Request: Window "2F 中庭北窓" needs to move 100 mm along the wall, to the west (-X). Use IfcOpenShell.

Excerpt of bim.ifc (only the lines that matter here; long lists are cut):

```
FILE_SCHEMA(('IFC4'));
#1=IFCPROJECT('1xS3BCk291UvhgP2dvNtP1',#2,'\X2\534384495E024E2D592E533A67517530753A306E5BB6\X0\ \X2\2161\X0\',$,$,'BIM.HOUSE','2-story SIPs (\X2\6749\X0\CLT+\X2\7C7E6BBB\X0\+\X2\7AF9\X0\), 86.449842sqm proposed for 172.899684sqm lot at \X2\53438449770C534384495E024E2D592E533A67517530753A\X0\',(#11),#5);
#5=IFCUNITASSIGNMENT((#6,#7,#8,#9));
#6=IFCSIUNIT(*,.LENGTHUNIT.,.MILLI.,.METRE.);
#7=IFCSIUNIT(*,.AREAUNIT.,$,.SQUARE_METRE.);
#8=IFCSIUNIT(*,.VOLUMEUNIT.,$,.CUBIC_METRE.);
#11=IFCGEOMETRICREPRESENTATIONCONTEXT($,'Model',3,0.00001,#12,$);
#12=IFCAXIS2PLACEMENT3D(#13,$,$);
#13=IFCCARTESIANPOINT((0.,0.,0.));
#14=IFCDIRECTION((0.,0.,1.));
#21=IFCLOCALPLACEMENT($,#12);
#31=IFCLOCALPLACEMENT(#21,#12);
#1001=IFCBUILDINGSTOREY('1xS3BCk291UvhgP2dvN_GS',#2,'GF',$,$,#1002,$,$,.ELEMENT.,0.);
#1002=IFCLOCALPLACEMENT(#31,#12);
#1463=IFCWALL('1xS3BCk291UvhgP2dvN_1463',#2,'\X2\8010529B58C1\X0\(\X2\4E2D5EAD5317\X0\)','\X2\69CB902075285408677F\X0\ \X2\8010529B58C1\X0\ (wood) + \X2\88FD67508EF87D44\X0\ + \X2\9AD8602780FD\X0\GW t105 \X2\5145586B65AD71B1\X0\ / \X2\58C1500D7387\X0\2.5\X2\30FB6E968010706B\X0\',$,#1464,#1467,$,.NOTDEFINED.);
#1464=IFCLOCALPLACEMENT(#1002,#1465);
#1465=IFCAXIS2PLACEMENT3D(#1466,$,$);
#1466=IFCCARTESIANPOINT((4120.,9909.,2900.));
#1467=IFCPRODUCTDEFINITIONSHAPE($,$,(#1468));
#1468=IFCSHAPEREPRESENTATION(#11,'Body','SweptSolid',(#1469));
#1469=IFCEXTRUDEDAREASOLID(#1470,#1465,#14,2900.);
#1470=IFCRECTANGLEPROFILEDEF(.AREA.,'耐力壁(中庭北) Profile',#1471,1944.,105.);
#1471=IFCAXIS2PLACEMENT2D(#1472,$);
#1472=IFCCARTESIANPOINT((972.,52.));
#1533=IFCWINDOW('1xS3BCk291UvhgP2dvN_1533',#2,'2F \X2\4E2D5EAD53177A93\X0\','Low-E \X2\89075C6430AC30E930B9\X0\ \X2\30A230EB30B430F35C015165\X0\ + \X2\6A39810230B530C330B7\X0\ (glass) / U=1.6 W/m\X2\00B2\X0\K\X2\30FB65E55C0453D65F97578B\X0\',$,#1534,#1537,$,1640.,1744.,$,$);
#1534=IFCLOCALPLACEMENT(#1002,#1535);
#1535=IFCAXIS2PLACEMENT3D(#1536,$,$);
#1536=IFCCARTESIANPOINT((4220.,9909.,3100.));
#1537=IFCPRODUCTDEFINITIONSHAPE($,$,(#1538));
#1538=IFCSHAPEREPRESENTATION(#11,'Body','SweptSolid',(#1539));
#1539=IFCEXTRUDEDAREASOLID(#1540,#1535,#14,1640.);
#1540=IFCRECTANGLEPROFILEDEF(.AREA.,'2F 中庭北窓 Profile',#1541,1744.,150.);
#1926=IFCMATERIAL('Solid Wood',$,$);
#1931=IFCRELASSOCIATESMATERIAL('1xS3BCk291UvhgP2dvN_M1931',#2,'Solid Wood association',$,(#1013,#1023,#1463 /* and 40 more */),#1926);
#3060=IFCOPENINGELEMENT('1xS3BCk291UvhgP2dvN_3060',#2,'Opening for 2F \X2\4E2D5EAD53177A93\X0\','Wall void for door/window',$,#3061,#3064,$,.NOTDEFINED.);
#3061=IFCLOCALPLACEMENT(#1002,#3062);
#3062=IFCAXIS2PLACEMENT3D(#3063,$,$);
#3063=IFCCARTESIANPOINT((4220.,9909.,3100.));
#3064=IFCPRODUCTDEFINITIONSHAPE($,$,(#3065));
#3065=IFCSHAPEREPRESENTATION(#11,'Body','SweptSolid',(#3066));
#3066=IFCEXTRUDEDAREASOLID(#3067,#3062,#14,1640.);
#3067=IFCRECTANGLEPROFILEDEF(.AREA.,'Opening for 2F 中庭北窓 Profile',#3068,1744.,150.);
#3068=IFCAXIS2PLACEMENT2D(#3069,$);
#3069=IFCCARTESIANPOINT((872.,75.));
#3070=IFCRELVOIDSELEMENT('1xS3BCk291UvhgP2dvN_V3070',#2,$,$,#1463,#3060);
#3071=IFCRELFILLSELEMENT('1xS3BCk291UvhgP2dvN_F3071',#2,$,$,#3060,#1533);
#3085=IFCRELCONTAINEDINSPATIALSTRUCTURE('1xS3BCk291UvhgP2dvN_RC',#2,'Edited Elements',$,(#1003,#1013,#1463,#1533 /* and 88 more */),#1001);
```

```python
import ifcopenshell
import ifcopenshell.api.geometry
import ifcopenshell.util.placement
import ifcopenshell.util.unit

model = ifcopenshell.open("bim.ifc")
unit_scale = ifcopenshell.util.unit.calculate_unit_scale(model)

window = model.by_guid("1xS3BCk291UvhgP2dvN_1533")
opening = window.FillsVoids[0].RelatingOpeningElement
wall = opening.VoidsElements[0].RelatingBuildingElement

wall_matrix = ifcopenshell.util.placement.get_local_placement(wall.ObjectPlacement)
shift = wall_matrix[:3, 0] * -0.1 / unit_scale
before = ifcopenshell.util.placement.get_local_placement(window.ObjectPlacement)[:3, 3].copy()

# The window is not placed relative to its opening, so move both.
for product in (opening, window):
    matrix = ifcopenshell.util.placement.get_local_placement(product.ObjectPlacement)
    matrix[:3, 3] += shift
    ifcopenshell.api.geometry.edit_object_placement(model, product=product, matrix=matrix, is_si=False)

after = ifcopenshell.util.placement.get_local_placement(window.ObjectPlacement)[:3, 3]
print("window moved by", (after - before).round(3) + 0.0)

model.write("bim-out.ifc")
```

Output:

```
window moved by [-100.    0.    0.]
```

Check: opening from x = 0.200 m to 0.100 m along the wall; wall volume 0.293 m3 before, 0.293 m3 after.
